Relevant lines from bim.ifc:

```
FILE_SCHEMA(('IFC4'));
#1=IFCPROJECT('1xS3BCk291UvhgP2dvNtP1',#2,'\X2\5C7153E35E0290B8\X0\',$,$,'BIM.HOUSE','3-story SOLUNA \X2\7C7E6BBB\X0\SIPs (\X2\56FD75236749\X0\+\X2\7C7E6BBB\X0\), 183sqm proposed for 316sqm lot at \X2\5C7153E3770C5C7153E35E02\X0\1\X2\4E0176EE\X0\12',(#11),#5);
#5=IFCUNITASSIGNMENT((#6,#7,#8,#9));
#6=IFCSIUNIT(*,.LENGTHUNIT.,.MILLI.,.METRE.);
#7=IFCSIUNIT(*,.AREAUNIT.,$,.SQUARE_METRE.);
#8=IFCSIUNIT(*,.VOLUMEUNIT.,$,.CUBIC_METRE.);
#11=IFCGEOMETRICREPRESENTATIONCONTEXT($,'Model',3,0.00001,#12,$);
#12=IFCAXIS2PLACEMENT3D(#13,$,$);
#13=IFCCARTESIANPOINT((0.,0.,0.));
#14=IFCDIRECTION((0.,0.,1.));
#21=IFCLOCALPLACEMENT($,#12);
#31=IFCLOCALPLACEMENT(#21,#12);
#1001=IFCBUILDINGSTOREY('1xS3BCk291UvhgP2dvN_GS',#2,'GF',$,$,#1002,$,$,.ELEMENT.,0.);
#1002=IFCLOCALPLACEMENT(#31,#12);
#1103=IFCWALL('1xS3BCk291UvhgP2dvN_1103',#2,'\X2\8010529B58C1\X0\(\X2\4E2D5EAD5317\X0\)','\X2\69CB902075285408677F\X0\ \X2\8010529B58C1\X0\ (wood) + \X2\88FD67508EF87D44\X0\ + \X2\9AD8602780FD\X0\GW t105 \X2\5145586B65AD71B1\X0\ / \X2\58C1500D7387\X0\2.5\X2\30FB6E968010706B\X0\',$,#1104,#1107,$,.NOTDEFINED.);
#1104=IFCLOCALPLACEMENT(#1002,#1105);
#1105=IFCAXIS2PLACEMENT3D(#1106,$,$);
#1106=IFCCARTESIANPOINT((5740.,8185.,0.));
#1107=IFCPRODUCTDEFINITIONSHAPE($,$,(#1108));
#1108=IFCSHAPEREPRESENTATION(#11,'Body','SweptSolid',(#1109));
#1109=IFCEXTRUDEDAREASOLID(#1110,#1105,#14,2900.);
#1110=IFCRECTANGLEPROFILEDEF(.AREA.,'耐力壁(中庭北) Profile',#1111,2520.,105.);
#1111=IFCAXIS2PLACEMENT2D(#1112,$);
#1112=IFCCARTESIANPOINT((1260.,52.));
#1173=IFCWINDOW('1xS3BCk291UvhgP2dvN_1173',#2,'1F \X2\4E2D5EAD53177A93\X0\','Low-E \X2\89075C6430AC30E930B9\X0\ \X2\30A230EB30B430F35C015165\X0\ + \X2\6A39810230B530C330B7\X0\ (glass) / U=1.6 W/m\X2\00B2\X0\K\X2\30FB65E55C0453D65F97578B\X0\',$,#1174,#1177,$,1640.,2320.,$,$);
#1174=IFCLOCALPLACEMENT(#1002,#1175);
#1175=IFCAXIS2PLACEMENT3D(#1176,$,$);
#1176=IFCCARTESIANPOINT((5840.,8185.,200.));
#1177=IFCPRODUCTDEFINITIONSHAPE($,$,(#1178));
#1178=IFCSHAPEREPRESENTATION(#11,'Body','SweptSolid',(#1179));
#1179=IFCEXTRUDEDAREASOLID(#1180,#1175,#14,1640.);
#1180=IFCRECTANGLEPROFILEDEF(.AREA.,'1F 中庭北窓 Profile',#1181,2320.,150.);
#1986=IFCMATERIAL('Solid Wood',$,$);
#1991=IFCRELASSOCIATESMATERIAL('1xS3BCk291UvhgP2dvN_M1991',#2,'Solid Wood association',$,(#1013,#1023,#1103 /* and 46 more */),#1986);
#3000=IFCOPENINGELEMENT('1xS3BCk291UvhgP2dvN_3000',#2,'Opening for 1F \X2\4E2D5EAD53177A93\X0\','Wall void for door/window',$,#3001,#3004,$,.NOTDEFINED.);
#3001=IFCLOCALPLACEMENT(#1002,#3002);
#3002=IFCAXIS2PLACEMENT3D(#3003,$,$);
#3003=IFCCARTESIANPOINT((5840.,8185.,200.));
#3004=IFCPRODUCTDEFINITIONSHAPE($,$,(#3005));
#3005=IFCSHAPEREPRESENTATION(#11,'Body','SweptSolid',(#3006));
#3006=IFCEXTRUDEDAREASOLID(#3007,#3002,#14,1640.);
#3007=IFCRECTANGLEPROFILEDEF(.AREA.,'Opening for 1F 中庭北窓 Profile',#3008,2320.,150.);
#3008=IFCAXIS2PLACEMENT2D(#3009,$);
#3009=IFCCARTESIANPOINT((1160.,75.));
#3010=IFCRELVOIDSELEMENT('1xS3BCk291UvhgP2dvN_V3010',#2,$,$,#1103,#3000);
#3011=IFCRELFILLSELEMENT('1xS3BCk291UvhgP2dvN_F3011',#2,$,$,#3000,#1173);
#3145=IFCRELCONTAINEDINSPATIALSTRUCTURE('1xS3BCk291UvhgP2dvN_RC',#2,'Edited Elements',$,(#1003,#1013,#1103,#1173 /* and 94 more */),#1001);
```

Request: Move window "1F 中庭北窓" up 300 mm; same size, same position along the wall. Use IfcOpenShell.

```python
import numpy as np
import ifcopenshell
import ifcopenshell.api.geometry
import ifcopenshell.util.placement
import ifcopenshell.util.unit

model = ifcopenshell.open("bim.ifc")
unit_scale = ifcopenshell.util.unit.calculate_unit_scale(model)

window = model.by_id(1173)
opening = window.FillsVoids[0].RelatingOpeningElement
dz = 0.3 / unit_scale

shift = np.array([0.0, 0.0, dz])
# The window is not placed relative to its opening, so move both.
for product in (opening, window):
    matrix = ifcopenshell.util.placement.get_local_placement(product.ObjectPlacement)
    matrix[:3, 3] += shift
    ifcopenshell.api.geometry.edit_object_placement(model, product=product, matrix=matrix, is_si=False)

print(f"moved by {dz * unit_scale:+.3f} m")

model.write("bim_edited.ifc")
```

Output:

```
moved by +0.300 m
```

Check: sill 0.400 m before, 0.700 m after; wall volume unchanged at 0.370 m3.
